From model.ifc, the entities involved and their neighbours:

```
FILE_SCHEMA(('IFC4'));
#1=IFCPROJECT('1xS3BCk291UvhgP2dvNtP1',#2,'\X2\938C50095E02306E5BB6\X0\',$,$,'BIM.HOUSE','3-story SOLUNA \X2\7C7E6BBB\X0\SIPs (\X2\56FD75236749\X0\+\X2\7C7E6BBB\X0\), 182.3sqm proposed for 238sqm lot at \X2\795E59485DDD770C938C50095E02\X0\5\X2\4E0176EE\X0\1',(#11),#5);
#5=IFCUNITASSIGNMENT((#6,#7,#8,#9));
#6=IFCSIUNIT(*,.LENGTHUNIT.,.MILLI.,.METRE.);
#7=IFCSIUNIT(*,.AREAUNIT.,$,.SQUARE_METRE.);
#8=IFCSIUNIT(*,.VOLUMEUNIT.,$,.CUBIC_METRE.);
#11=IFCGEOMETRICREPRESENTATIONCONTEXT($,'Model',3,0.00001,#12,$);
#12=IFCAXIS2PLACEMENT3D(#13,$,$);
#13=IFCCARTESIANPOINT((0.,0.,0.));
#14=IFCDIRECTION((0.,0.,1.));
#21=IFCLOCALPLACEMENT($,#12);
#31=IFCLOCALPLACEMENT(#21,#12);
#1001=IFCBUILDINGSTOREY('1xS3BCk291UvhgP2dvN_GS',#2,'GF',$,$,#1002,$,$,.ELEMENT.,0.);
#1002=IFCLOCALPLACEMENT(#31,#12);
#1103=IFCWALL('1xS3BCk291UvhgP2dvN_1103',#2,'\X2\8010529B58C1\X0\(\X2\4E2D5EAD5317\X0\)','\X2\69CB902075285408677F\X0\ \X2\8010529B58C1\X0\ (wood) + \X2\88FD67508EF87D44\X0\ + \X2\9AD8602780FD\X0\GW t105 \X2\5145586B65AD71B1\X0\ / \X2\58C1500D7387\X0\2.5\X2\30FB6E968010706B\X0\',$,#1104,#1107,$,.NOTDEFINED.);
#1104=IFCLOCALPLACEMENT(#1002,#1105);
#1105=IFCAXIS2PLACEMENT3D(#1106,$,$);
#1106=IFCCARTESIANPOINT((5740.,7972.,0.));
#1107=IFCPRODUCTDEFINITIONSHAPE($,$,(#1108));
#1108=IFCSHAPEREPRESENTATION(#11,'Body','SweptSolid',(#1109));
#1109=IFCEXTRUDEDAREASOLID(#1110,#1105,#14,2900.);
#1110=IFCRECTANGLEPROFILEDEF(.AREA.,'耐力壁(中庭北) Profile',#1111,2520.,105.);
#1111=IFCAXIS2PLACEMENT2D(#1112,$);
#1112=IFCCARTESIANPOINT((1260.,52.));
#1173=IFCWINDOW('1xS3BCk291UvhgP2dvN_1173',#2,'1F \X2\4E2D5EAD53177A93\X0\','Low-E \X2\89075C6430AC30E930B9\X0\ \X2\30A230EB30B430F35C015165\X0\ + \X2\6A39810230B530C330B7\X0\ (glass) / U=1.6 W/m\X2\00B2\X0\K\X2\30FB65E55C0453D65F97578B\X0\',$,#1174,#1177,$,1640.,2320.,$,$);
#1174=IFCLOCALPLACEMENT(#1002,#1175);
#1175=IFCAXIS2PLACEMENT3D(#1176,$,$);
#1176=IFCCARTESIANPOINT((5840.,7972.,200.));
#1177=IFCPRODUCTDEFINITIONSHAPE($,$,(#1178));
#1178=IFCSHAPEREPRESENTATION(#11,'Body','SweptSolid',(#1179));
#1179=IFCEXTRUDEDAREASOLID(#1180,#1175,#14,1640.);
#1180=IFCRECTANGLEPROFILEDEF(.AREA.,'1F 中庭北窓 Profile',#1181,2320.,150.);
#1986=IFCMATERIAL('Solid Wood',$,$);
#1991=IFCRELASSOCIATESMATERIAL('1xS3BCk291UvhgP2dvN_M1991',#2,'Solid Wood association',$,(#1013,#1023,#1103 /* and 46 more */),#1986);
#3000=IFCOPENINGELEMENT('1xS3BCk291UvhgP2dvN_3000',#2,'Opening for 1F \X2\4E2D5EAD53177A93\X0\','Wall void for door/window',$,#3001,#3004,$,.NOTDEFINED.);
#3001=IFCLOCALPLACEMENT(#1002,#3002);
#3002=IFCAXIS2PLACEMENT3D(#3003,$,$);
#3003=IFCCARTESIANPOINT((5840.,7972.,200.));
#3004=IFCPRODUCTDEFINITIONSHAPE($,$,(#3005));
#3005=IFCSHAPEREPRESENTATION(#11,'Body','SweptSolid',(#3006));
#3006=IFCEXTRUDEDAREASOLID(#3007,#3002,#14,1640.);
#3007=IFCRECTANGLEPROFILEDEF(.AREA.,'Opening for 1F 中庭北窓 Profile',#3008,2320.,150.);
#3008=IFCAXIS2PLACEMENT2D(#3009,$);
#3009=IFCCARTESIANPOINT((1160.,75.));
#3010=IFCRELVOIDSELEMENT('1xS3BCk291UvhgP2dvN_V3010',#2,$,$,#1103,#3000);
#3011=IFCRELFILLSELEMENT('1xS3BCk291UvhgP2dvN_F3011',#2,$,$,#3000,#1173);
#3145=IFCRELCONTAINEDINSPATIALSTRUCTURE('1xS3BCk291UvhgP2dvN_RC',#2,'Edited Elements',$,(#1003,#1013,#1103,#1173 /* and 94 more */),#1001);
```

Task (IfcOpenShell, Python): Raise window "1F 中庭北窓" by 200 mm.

```python
import numpy as np
import ifcopenshell
import ifcopenshell.api.geometry
import ifcopenshell.util.placement
import ifcopenshell.util.unit

model = ifcopenshell.open("model.ifc")
unit_scale = ifcopenshell.util.unit.calculate_unit_scale(model)

window = model.by_id(1173)
opening = window.FillsVoids[0].RelatingOpeningElement
dz = 0.2 / unit_scale

shift = np.array([0.0, 0.0, dz])
# The window is not placed relative to its opening, so move both.
for product in (opening, window):
    matrix = ifcopenshell.util.placement.get_local_placement(product.ObjectPlacement)
    matrix[:3, 3] += shift
    ifcopenshell.api.geometry.edit_object_placement(model, product=product, matrix=matrix, is_si=False)

print(f"moved by {dz * unit_scale:+.3f} m")

model.write("model_rev.ifc")
```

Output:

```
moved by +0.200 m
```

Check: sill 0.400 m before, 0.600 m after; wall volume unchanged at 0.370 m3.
